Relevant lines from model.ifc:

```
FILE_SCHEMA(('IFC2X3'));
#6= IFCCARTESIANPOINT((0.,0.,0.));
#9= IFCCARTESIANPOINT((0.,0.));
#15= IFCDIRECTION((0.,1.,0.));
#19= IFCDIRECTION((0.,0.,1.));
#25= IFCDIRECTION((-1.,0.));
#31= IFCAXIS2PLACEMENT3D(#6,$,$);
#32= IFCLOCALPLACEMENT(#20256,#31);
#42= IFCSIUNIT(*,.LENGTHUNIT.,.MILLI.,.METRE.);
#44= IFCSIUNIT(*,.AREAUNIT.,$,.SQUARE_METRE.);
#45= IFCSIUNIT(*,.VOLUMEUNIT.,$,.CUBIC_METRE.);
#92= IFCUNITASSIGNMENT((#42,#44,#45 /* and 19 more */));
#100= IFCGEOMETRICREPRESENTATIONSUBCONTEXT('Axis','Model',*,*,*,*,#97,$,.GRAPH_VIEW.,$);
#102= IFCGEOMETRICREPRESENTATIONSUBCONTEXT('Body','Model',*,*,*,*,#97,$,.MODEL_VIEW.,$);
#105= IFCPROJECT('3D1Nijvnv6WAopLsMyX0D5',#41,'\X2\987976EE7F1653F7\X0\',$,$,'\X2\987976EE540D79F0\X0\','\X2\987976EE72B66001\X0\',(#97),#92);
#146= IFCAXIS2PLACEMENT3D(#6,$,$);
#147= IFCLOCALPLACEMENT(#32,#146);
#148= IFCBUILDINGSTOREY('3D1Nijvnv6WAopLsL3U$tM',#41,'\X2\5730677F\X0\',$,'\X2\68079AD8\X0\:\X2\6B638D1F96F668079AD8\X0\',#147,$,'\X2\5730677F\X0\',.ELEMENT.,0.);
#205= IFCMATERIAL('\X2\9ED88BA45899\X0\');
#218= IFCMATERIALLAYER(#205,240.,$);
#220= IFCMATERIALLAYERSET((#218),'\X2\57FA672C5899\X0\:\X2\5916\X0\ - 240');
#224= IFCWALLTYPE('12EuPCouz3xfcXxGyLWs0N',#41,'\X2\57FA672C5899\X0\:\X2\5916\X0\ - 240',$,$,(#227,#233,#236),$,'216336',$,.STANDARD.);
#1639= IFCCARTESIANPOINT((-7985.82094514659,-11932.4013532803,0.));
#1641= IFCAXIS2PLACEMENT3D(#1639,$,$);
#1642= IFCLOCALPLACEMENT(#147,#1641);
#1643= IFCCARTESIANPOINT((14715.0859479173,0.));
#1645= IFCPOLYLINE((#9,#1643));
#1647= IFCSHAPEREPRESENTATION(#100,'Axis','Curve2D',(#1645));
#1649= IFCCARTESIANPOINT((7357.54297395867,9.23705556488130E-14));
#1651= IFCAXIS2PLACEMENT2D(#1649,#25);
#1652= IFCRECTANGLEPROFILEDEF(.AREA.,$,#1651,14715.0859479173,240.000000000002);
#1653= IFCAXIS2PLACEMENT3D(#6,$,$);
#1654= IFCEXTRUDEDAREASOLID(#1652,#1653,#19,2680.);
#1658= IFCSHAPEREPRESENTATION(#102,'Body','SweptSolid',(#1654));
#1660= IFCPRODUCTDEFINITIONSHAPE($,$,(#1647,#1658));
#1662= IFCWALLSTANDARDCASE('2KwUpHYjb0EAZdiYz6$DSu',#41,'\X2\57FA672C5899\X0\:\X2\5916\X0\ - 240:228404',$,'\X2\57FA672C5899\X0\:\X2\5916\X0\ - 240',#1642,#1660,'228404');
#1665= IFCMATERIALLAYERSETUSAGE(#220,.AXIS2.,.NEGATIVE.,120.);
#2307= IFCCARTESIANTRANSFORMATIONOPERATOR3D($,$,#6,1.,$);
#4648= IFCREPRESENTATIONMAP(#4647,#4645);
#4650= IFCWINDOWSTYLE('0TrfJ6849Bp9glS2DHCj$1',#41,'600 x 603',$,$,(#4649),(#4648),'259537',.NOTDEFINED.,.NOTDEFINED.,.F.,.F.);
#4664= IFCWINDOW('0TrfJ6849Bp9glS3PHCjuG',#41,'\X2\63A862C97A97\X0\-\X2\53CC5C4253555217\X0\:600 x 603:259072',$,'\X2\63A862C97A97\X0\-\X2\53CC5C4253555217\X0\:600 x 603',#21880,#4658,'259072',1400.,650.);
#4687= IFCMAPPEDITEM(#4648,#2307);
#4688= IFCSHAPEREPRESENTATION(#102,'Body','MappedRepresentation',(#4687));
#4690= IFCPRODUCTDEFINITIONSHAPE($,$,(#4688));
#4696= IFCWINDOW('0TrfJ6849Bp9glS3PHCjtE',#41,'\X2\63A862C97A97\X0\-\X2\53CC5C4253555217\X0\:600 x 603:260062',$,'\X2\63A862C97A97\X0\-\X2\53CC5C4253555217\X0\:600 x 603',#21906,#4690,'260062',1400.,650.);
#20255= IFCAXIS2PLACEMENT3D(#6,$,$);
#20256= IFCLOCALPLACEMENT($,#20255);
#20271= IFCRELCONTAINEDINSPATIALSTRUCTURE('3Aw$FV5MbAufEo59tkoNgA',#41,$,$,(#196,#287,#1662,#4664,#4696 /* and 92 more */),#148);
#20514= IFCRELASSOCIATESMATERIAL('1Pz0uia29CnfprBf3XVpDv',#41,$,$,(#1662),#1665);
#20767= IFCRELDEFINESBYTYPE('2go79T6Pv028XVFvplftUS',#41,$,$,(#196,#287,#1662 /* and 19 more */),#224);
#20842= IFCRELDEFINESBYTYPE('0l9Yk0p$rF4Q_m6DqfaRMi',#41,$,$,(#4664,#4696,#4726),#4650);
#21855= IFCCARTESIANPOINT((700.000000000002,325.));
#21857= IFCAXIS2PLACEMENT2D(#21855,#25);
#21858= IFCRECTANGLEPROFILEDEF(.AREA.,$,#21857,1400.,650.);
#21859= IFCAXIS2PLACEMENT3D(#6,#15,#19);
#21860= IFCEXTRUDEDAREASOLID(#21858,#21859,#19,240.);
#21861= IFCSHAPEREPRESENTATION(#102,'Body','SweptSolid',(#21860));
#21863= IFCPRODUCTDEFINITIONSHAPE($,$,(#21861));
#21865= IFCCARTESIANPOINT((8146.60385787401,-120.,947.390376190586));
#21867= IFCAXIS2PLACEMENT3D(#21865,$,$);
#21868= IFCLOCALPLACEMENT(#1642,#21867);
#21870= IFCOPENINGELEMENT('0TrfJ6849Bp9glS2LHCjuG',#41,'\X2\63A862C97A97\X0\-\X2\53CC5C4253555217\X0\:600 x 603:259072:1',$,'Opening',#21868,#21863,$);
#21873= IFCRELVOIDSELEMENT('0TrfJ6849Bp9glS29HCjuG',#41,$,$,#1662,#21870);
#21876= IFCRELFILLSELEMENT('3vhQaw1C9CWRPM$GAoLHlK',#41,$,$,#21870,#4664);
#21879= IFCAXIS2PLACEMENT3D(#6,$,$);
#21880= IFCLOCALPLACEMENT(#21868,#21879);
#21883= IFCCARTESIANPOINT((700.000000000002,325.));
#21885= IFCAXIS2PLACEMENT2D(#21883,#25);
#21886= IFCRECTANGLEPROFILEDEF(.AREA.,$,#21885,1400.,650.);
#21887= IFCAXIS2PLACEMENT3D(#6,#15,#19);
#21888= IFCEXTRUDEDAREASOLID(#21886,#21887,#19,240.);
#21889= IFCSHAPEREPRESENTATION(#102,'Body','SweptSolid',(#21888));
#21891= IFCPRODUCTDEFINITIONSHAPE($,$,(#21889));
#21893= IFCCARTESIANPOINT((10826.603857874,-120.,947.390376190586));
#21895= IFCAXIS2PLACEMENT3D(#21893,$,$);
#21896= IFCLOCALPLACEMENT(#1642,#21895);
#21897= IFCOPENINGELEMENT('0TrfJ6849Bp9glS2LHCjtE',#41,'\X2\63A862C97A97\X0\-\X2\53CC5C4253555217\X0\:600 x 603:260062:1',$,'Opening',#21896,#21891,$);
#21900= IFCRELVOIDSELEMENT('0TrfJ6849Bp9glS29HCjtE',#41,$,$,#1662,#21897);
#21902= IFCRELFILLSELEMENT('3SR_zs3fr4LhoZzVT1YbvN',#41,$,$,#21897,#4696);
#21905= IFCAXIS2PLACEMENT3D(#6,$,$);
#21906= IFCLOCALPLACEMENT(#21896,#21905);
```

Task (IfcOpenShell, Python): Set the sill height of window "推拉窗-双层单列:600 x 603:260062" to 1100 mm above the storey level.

```python
import numpy as np
import ifcopenshell
import ifcopenshell.api.geometry
import ifcopenshell.geom
import ifcopenshell.util.element
import ifcopenshell.util.placement
import ifcopenshell.util.shape
import ifcopenshell.util.unit

model = ifcopenshell.open("model.ifc")
unit_scale = ifcopenshell.util.unit.calculate_unit_scale(model)

window = model.by_guid("0TrfJ6849Bp9glS3PHCjtE")
opening = window.FillsVoids[0].RelatingOpeningElement
storey = ifcopenshell.util.element.get_container(window, ifc_class="IfcBuildingStorey")
level = ifcopenshell.util.placement.get_local_placement(storey.ObjectPlacement)[2, 3]

# The opening's origin need not be at the sill, so measure its lowest point.
shape = ifcopenshell.geom.create_shape(ifcopenshell.geom.settings(), opening)
bottom = ifcopenshell.util.shape.get_shape_bottom_elevation(shape, shape.geometry) / unit_scale
dz = level + 1100.0 - bottom

shift = np.array([0.0, 0.0, dz])
# The window is placed relative to its opening, so it follows when the opening moves.
matrix = ifcopenshell.util.placement.get_local_placement(opening.ObjectPlacement)
matrix[:3, 3] += shift
ifcopenshell.api.geometry.edit_object_placement(
    model, product=opening, matrix=matrix, is_si=False, should_transform_children=True
)

print(f"moved by {dz * unit_scale:+.3f} m")

model.write("model_v2.ifc")
```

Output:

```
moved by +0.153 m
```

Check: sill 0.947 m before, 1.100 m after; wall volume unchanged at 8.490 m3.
